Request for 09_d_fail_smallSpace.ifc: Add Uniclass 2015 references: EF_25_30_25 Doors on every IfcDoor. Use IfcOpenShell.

First a look at what the model holds.

```python
import ifcopenshell

model = ifcopenshell.open("09_d_fail_smallSpace.ifc")
print(model.schema)
print("classifications:", [c.Name for c in model.by_type("IfcClassification")])
for ifc_class in ("IfcDoor", "IfcRoof", "IfcStair", "IfcWall", "IfcWindow"):
    print(ifc_class, len(model.by_type(ifc_class)))
```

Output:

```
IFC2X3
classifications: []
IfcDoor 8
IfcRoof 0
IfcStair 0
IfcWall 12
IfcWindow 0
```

```python
import ifcopenshell
import ifcopenshell.api.classification

model = ifcopenshell.open("09_d_fail_smallSpace.ifc")

# IFC2X3 requires Source and Edition and has no link from the project to the system.
system = model.create_entity("IfcClassification", Source="NBS", Edition="2015", Name="Uniclass 2015")

codes = {
    "IfcDoor": ("EF_25_30_25", "Doors"),
}
for ifc_class, (code, name) in codes.items():
    products = model.by_type(ifc_class)
    ifcopenshell.api.classification.add_reference(
        model, products=products, classification=system, identification=code, name=name
    )
    print(code, len(products))

model.write("09_d_fail_smallSpace_rev.ifc")
```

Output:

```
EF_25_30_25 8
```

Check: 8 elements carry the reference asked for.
